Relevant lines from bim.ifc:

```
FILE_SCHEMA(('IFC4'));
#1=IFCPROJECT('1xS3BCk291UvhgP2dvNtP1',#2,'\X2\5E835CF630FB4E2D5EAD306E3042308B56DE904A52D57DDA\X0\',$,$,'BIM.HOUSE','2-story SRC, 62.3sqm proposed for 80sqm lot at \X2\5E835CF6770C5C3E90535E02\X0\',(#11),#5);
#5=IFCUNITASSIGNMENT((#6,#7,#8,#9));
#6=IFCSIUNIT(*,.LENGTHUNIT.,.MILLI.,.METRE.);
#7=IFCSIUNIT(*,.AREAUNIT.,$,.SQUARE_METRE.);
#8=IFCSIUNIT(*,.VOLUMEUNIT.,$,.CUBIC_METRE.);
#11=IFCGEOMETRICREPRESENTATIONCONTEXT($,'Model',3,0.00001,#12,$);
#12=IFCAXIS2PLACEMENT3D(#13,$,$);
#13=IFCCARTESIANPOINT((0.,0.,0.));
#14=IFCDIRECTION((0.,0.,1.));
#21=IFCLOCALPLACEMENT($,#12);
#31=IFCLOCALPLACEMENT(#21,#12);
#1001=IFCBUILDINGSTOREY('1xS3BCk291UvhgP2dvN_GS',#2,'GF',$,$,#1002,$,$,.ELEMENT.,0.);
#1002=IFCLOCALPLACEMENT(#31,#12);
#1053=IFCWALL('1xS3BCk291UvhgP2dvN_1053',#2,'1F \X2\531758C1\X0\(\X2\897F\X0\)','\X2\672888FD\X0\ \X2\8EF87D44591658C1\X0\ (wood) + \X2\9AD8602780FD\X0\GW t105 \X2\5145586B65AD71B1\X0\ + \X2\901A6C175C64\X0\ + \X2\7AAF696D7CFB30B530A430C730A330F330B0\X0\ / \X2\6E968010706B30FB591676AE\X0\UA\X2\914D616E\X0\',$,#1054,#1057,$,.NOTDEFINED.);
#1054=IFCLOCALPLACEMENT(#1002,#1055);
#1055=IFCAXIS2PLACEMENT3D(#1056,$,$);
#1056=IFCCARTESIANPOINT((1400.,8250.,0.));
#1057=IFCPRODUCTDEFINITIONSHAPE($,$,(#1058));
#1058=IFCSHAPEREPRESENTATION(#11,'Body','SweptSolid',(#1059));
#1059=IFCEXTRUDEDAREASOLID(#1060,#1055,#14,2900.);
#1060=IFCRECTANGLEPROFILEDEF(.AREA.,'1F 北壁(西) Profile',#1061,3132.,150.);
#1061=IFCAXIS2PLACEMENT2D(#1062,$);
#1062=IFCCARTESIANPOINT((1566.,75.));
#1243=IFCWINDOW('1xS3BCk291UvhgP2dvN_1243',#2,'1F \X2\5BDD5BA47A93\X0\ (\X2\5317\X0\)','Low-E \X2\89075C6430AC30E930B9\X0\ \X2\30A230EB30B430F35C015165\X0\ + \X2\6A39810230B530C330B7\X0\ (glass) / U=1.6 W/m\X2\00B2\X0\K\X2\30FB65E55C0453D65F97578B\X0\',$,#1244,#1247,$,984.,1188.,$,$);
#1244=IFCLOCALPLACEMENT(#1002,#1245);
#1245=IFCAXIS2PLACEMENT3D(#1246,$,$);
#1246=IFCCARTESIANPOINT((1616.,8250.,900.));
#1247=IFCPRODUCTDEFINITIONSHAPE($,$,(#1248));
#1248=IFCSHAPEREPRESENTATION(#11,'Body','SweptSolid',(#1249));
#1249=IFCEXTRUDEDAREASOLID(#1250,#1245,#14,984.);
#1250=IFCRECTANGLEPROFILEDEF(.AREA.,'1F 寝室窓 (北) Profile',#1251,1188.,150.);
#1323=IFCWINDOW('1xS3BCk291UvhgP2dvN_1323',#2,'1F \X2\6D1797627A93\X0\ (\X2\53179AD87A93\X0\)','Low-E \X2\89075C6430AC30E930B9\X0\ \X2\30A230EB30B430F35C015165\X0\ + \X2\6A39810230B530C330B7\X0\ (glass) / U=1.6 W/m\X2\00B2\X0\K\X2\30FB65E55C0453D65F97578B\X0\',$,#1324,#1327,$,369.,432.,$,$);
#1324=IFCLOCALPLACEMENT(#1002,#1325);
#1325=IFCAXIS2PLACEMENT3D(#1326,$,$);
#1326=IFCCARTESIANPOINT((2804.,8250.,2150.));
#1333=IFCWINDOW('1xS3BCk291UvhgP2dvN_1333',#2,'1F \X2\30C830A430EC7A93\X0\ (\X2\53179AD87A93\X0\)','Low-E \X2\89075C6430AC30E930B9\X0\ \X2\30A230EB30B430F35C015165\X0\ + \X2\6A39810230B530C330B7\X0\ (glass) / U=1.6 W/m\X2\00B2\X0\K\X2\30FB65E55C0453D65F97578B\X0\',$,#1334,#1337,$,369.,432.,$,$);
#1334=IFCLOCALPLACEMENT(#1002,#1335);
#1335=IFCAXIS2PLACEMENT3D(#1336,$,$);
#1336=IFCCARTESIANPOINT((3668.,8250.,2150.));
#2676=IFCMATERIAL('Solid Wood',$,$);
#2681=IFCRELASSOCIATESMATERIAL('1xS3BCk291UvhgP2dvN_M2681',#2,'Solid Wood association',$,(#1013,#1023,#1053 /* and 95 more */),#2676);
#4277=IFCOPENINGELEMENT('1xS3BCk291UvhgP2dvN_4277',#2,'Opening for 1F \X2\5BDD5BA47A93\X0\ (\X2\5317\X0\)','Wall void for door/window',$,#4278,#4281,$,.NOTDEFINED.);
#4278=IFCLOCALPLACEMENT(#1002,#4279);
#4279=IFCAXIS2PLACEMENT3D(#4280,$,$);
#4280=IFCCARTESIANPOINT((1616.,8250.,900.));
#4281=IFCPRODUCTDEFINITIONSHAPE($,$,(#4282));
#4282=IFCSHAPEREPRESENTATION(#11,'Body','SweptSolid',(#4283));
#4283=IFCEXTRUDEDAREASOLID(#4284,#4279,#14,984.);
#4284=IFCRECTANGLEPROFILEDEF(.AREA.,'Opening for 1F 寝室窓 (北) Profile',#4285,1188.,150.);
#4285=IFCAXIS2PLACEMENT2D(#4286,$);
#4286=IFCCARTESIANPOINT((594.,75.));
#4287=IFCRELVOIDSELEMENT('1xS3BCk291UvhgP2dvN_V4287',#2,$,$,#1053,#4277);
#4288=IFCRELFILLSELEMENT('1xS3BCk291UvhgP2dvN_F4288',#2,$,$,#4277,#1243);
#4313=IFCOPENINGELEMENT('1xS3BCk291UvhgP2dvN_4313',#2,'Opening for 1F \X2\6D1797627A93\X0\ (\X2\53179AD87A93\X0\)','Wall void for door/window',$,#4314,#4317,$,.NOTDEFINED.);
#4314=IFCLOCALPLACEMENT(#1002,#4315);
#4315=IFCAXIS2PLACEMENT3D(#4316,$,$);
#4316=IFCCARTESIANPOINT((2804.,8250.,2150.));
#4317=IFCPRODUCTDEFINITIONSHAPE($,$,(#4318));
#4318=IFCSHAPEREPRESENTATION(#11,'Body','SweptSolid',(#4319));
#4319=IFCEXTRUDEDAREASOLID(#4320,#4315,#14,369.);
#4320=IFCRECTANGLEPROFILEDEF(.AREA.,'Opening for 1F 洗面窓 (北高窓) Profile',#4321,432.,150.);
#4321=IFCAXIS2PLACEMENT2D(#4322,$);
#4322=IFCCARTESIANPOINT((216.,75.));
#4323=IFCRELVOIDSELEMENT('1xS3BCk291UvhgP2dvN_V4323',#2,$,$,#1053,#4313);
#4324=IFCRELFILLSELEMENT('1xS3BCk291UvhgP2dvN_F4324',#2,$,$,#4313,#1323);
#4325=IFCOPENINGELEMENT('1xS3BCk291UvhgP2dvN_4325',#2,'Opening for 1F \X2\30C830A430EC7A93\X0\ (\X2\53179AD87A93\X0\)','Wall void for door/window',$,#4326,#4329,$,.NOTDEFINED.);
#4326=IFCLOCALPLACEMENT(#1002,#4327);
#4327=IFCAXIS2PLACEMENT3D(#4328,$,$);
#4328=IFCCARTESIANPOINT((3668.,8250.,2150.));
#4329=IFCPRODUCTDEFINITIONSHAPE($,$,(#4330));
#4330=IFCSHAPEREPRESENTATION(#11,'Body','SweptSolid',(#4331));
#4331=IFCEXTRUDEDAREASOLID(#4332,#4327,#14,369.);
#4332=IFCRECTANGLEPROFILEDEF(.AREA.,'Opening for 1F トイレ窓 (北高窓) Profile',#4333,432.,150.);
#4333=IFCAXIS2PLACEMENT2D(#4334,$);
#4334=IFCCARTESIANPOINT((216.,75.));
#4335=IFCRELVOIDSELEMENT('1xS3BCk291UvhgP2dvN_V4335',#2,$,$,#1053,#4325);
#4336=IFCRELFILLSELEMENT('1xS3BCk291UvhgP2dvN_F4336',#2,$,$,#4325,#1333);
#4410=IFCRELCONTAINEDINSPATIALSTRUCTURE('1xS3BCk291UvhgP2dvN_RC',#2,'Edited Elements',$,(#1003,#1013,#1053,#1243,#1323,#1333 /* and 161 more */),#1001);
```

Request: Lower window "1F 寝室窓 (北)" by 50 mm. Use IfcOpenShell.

```python
import numpy as np
import ifcopenshell
import ifcopenshell.api.geometry
import ifcopenshell.util.placement
import ifcopenshell.util.unit

model = ifcopenshell.open("bim.ifc")
unit_scale = ifcopenshell.util.unit.calculate_unit_scale(model)

window = model.by_id(1243)
opening = window.FillsVoids[0].RelatingOpeningElement
dz = -0.05 / unit_scale

shift = np.array([0.0, 0.0, dz])
# The window is not placed relative to its opening, so move both.
for product in (opening, window):
    matrix = ifcopenshell.util.placement.get_local_placement(product.ObjectPlacement)
    matrix[:3, 3] += shift
    ifcopenshell.api.geometry.edit_object_placement(model, product=product, matrix=matrix, is_si=False)

print(f"moved by {dz * unit_scale:+.3f} m")

model.write("bim_v2.ifc")
```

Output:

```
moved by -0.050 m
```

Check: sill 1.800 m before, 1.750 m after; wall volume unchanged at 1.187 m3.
